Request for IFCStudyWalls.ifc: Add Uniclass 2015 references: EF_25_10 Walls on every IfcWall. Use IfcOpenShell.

First a look at what the model holds.

```python
import ifcopenshell

model = ifcopenshell.open("IFCStudyWalls.ifc")
print(model.schema)
print("classifications:", [c.Name for c in model.by_type("IfcClassification")])
for ifc_class in ("IfcDoor", "IfcRoof", "IfcStair", "IfcWall", "IfcWindow"):
    print(ifc_class, len(model.by_type(ifc_class)))
```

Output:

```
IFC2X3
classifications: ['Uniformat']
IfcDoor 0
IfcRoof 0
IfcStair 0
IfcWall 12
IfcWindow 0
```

```python
import ifcopenshell
import ifcopenshell.api.classification

model = ifcopenshell.open("IFCStudyWalls.ifc")

# IFC2X3 requires Source and Edition and has no link from the project to the system.
system = model.create_entity("IfcClassification", Source="NBS", Edition="2015", Name="Uniclass 2015")

codes = {
    "IfcWall": ("EF_25_10", "Walls"),
}
for ifc_class, (code, name) in codes.items():
    products = model.by_type(ifc_class)
    ifcopenshell.api.classification.add_reference(
        model, products=products, classification=system, identification=code, name=name
    )
    print(code, len(products))

model.write("IFCStudyWalls-out.ifc")
```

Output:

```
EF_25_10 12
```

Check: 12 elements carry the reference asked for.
